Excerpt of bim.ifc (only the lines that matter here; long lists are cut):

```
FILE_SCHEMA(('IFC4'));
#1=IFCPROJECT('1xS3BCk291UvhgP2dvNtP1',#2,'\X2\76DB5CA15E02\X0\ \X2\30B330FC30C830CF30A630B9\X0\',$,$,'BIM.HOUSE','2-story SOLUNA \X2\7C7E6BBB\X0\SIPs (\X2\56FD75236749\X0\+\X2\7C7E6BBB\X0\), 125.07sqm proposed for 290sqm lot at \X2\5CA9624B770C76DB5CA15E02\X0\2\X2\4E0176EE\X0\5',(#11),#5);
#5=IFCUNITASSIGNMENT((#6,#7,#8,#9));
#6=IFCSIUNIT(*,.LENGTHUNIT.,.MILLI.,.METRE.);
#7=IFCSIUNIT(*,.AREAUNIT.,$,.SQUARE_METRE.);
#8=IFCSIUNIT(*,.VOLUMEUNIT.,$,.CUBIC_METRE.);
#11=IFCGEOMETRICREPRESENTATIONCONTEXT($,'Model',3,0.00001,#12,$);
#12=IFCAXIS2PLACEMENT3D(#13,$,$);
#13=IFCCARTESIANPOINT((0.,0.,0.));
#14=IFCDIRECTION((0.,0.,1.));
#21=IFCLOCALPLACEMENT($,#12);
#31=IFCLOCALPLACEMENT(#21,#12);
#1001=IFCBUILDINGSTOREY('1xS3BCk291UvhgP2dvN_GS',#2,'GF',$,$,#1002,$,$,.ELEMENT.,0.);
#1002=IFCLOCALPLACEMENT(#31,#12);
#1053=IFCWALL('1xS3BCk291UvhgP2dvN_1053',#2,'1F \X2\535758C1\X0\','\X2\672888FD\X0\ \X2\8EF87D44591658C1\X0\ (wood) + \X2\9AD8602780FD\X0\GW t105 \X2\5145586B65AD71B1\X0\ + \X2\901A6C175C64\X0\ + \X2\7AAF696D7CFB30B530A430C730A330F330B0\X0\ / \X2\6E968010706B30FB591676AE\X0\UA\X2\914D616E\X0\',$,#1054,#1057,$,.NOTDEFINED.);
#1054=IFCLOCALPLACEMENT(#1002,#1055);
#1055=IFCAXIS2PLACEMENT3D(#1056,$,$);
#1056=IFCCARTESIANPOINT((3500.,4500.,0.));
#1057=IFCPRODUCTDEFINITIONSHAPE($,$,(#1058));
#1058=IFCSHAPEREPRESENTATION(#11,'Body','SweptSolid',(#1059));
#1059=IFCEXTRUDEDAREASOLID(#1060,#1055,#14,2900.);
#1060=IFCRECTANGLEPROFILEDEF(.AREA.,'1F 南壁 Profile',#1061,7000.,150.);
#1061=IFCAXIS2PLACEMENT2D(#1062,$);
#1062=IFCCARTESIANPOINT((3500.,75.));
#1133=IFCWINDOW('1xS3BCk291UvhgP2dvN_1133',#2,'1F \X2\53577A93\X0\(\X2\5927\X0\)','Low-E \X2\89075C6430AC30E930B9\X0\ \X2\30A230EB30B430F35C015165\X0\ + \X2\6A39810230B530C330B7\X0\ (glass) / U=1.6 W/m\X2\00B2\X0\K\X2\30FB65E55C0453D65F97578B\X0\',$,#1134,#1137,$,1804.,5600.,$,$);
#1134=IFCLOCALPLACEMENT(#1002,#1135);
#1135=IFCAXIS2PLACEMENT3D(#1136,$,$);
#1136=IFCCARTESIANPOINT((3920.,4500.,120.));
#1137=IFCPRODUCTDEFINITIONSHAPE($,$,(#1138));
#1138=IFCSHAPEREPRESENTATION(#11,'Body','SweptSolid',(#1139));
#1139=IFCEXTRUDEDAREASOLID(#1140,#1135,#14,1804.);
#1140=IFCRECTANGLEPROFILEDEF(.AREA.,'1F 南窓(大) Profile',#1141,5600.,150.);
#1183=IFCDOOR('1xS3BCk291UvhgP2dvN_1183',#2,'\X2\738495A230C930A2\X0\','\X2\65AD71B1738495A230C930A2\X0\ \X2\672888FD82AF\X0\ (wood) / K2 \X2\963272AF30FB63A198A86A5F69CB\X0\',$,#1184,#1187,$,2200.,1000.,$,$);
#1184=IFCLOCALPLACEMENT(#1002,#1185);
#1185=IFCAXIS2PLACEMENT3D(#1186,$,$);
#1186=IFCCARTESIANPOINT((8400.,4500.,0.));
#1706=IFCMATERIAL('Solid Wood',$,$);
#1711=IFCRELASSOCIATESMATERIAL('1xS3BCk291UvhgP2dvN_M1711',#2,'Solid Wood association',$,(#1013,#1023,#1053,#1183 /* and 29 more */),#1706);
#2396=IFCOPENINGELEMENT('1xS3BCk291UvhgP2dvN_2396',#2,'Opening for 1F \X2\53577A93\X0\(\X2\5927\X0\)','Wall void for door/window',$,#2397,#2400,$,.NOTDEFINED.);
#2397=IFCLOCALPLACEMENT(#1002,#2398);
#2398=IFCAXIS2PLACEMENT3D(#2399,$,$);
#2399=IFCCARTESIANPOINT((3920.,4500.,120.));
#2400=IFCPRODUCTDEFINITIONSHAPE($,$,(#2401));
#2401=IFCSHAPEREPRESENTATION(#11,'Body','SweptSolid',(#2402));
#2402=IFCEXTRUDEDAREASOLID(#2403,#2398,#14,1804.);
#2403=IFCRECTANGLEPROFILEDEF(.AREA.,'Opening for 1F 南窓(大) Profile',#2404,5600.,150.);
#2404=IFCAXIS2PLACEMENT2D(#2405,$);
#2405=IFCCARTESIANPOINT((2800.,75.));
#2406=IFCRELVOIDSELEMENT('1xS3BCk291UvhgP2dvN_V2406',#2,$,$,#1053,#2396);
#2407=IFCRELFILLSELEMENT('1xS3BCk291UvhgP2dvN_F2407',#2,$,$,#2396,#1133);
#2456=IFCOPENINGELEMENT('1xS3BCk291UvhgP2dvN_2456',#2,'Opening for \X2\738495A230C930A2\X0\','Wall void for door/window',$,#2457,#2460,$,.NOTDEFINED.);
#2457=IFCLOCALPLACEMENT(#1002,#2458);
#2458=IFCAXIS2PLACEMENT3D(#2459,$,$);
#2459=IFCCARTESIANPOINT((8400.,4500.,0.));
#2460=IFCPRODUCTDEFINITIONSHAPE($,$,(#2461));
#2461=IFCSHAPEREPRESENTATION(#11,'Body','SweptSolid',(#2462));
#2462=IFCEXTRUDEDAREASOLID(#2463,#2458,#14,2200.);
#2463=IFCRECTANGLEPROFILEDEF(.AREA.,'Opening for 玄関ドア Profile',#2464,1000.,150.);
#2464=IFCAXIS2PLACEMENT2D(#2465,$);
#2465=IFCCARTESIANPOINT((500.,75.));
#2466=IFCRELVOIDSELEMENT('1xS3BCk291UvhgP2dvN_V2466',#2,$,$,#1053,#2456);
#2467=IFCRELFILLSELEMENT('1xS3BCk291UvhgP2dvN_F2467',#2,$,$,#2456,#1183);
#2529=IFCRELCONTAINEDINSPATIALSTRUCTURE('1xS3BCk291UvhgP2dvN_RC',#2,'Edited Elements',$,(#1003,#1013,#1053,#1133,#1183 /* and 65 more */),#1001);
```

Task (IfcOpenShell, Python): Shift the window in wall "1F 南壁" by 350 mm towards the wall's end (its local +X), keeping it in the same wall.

```python
import ifcopenshell
import ifcopenshell.api.geometry
import ifcopenshell.util.placement

model = ifcopenshell.open("bim.ifc")

window = model.by_guid("1xS3BCk291UvhgP2dvN_1133")
opening = window.FillsVoids[0].RelatingOpeningElement
wall = opening.VoidsElements[0].RelatingBuildingElement

wall_matrix = ifcopenshell.util.placement.get_local_placement(wall.ObjectPlacement)
shift = wall_matrix[:3, 0] * 350.0
before = ifcopenshell.util.placement.get_local_placement(window.ObjectPlacement)[:3, 3].copy()

# The window is not placed relative to its opening, so move both.
for product in (opening, window):
    matrix = ifcopenshell.util.placement.get_local_placement(product.ObjectPlacement)
    matrix[:3, 3] += shift
    ifcopenshell.api.geometry.edit_object_placement(model, product=product, matrix=matrix, is_si=False)

after = ifcopenshell.util.placement.get_local_placement(window.ObjectPlacement)[:3, 3]
print("window moved by", (after - before).round(3) + 0.0)

model.write("bim_edited.ifc")
```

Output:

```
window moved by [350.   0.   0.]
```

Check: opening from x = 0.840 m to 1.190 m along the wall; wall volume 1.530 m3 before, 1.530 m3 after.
